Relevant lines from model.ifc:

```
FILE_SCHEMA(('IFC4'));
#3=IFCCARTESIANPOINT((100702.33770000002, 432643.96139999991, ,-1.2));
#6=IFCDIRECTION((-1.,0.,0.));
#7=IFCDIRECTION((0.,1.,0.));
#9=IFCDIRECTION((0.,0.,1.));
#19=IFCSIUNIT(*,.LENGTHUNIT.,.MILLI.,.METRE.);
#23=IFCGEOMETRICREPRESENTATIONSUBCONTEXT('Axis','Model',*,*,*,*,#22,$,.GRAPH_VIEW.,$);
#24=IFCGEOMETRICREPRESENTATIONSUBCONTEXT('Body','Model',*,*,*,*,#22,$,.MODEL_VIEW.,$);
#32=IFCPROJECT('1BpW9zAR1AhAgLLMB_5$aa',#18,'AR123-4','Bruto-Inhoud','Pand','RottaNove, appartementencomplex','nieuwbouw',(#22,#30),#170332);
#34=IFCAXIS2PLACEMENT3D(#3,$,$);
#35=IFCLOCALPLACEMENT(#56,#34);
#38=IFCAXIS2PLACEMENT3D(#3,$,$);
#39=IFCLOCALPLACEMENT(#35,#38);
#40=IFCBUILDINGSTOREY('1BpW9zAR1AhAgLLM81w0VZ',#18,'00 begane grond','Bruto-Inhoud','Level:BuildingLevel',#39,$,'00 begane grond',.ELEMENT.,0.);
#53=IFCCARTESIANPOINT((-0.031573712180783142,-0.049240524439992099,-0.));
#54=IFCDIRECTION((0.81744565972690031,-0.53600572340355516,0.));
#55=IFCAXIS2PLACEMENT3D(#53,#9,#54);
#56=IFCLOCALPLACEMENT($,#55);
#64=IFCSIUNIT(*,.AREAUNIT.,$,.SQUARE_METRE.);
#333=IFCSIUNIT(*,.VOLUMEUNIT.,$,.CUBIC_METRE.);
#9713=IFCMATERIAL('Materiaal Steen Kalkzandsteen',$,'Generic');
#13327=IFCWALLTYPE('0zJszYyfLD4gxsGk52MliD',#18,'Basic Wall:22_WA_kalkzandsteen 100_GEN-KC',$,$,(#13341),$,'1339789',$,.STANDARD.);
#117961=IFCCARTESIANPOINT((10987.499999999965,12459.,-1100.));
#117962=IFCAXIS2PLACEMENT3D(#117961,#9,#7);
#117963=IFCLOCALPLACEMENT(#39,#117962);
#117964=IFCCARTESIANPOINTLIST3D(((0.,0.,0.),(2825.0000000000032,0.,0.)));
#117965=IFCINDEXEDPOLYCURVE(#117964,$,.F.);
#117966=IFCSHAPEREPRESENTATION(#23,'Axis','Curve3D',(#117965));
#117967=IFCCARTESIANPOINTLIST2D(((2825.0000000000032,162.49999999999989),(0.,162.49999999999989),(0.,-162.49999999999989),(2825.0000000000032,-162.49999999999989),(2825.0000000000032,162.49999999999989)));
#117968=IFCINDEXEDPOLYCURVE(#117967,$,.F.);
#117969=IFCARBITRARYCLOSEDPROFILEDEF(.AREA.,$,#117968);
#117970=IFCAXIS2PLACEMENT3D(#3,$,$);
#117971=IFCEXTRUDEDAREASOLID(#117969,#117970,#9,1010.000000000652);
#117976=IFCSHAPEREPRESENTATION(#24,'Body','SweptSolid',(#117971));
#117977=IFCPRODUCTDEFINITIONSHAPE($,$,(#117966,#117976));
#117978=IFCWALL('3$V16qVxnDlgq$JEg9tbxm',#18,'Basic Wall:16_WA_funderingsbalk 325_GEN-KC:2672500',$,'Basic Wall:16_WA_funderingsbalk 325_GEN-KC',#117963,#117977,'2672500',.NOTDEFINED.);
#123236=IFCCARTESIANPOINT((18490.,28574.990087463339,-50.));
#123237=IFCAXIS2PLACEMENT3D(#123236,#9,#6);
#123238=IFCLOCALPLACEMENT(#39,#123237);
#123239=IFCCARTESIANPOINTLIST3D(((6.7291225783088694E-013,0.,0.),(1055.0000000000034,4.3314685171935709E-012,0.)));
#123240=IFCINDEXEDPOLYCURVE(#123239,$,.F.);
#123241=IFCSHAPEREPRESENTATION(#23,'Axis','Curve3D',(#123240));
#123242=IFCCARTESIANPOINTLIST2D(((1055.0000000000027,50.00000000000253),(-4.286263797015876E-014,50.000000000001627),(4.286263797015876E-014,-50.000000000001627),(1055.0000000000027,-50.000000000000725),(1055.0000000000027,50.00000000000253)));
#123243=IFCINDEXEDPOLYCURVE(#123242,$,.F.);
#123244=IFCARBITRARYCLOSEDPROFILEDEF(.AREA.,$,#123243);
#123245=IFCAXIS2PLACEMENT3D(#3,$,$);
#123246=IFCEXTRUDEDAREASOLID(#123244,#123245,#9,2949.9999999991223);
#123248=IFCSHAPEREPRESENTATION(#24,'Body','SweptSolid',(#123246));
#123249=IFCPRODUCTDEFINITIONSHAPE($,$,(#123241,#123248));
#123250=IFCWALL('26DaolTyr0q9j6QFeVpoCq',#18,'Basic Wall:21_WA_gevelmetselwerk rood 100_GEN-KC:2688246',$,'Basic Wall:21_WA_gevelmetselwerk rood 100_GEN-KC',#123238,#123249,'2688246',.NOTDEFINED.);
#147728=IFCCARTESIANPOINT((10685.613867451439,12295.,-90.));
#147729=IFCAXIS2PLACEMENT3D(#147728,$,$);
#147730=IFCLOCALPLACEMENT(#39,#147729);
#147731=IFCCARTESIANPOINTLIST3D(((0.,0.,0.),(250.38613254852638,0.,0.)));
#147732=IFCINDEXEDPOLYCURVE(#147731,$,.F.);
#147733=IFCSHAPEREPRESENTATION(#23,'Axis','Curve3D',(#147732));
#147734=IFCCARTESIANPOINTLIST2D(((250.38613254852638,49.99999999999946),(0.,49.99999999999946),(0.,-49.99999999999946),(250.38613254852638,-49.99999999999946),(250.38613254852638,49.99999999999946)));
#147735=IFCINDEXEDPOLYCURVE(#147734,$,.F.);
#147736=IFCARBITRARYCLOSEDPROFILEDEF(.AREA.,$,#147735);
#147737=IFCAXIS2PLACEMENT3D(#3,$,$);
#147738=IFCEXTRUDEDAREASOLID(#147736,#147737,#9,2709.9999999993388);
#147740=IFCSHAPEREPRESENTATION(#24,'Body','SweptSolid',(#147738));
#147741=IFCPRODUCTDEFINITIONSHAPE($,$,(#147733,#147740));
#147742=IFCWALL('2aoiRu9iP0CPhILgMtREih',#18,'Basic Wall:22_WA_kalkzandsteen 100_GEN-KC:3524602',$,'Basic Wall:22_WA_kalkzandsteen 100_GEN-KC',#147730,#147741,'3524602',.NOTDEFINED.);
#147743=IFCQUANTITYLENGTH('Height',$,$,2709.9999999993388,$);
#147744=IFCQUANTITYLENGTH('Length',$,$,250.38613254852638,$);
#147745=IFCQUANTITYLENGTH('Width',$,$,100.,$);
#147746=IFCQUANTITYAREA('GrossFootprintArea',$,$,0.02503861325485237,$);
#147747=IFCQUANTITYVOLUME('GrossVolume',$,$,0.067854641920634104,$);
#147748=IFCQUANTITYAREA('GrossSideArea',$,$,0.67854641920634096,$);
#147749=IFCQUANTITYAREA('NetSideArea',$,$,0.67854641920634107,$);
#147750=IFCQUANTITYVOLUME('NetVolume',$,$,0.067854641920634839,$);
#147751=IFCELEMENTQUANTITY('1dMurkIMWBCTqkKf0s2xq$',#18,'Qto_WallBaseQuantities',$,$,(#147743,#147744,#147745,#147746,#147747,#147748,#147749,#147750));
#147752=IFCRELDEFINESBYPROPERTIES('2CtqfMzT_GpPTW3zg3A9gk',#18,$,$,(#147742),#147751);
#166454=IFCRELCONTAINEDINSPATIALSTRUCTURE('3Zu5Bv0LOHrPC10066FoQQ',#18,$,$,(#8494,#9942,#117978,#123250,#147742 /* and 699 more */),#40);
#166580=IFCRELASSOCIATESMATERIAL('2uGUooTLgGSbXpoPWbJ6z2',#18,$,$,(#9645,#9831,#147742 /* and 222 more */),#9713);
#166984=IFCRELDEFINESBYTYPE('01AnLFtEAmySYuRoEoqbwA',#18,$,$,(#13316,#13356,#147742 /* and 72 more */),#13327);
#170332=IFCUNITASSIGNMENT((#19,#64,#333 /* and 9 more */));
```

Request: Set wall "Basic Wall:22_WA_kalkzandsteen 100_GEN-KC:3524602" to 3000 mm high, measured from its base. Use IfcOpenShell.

```python
import ifcopenshell
import ifcopenshell.api.pset
import ifcopenshell.geom
import ifcopenshell.util.element
import ifcopenshell.util.representation
import ifcopenshell.util.shape
import ifcopenshell.util.unit

model = ifcopenshell.open("model.ifc")
unit_scale = ifcopenshell.util.unit.calculate_unit_scale(model)
area_scale = ifcopenshell.util.unit.calculate_unit_scale(model, "AREAUNIT")
volume_scale = ifcopenshell.util.unit.calculate_unit_scale(model, "VOLUMEUNIT")
settings = ifcopenshell.geom.settings()


def volume(element):
    """Net volume in cubic metres, openings subtracted."""
    shape = ifcopenshell.geom.create_shape(settings, element)
    return ifcopenshell.util.shape.get_volume(shape.geometry)


wall = model.by_guid("2aoiRu9iP0CPhILgMtREih")
before = volume(wall)

body = ifcopenshell.util.representation.get_representation(wall, "Model", "Body")
solid = body.Items[0]
old_height = solid.Depth
solid.Depth = 3 / unit_scale
after = volume(wall)
thickness = 0.1  # wall thickness in metres

# Update the stored height, areas and volumes.
qto = model.by_id(ifcopenshell.util.element.get_pset(wall, "Qto_WallBaseQuantities", should_inherit=False)["id"])
ifcopenshell.api.pset.edit_qto(model, qto=qto, properties={
    "Height": solid.Depth,
    "GrossVolume": ifcopenshell.util.element.get_pset(wall, "Qto_WallBaseQuantities", "GrossVolume") * solid.Depth / old_height,
    "GrossSideArea": ifcopenshell.util.element.get_pset(wall, "Qto_WallBaseQuantities", "GrossSideArea") * solid.Depth / old_height,
    "NetSideArea": after / thickness / area_scale,
    "NetVolume": after / volume_scale,
})

print(f"height {old_height:g} -> {solid.Depth:g}, volume {before:.3f} -> {after:.3f} m3")

model.write("model_edited.ifc")
```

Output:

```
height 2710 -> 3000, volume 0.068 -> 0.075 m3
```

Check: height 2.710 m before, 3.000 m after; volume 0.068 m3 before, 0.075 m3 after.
